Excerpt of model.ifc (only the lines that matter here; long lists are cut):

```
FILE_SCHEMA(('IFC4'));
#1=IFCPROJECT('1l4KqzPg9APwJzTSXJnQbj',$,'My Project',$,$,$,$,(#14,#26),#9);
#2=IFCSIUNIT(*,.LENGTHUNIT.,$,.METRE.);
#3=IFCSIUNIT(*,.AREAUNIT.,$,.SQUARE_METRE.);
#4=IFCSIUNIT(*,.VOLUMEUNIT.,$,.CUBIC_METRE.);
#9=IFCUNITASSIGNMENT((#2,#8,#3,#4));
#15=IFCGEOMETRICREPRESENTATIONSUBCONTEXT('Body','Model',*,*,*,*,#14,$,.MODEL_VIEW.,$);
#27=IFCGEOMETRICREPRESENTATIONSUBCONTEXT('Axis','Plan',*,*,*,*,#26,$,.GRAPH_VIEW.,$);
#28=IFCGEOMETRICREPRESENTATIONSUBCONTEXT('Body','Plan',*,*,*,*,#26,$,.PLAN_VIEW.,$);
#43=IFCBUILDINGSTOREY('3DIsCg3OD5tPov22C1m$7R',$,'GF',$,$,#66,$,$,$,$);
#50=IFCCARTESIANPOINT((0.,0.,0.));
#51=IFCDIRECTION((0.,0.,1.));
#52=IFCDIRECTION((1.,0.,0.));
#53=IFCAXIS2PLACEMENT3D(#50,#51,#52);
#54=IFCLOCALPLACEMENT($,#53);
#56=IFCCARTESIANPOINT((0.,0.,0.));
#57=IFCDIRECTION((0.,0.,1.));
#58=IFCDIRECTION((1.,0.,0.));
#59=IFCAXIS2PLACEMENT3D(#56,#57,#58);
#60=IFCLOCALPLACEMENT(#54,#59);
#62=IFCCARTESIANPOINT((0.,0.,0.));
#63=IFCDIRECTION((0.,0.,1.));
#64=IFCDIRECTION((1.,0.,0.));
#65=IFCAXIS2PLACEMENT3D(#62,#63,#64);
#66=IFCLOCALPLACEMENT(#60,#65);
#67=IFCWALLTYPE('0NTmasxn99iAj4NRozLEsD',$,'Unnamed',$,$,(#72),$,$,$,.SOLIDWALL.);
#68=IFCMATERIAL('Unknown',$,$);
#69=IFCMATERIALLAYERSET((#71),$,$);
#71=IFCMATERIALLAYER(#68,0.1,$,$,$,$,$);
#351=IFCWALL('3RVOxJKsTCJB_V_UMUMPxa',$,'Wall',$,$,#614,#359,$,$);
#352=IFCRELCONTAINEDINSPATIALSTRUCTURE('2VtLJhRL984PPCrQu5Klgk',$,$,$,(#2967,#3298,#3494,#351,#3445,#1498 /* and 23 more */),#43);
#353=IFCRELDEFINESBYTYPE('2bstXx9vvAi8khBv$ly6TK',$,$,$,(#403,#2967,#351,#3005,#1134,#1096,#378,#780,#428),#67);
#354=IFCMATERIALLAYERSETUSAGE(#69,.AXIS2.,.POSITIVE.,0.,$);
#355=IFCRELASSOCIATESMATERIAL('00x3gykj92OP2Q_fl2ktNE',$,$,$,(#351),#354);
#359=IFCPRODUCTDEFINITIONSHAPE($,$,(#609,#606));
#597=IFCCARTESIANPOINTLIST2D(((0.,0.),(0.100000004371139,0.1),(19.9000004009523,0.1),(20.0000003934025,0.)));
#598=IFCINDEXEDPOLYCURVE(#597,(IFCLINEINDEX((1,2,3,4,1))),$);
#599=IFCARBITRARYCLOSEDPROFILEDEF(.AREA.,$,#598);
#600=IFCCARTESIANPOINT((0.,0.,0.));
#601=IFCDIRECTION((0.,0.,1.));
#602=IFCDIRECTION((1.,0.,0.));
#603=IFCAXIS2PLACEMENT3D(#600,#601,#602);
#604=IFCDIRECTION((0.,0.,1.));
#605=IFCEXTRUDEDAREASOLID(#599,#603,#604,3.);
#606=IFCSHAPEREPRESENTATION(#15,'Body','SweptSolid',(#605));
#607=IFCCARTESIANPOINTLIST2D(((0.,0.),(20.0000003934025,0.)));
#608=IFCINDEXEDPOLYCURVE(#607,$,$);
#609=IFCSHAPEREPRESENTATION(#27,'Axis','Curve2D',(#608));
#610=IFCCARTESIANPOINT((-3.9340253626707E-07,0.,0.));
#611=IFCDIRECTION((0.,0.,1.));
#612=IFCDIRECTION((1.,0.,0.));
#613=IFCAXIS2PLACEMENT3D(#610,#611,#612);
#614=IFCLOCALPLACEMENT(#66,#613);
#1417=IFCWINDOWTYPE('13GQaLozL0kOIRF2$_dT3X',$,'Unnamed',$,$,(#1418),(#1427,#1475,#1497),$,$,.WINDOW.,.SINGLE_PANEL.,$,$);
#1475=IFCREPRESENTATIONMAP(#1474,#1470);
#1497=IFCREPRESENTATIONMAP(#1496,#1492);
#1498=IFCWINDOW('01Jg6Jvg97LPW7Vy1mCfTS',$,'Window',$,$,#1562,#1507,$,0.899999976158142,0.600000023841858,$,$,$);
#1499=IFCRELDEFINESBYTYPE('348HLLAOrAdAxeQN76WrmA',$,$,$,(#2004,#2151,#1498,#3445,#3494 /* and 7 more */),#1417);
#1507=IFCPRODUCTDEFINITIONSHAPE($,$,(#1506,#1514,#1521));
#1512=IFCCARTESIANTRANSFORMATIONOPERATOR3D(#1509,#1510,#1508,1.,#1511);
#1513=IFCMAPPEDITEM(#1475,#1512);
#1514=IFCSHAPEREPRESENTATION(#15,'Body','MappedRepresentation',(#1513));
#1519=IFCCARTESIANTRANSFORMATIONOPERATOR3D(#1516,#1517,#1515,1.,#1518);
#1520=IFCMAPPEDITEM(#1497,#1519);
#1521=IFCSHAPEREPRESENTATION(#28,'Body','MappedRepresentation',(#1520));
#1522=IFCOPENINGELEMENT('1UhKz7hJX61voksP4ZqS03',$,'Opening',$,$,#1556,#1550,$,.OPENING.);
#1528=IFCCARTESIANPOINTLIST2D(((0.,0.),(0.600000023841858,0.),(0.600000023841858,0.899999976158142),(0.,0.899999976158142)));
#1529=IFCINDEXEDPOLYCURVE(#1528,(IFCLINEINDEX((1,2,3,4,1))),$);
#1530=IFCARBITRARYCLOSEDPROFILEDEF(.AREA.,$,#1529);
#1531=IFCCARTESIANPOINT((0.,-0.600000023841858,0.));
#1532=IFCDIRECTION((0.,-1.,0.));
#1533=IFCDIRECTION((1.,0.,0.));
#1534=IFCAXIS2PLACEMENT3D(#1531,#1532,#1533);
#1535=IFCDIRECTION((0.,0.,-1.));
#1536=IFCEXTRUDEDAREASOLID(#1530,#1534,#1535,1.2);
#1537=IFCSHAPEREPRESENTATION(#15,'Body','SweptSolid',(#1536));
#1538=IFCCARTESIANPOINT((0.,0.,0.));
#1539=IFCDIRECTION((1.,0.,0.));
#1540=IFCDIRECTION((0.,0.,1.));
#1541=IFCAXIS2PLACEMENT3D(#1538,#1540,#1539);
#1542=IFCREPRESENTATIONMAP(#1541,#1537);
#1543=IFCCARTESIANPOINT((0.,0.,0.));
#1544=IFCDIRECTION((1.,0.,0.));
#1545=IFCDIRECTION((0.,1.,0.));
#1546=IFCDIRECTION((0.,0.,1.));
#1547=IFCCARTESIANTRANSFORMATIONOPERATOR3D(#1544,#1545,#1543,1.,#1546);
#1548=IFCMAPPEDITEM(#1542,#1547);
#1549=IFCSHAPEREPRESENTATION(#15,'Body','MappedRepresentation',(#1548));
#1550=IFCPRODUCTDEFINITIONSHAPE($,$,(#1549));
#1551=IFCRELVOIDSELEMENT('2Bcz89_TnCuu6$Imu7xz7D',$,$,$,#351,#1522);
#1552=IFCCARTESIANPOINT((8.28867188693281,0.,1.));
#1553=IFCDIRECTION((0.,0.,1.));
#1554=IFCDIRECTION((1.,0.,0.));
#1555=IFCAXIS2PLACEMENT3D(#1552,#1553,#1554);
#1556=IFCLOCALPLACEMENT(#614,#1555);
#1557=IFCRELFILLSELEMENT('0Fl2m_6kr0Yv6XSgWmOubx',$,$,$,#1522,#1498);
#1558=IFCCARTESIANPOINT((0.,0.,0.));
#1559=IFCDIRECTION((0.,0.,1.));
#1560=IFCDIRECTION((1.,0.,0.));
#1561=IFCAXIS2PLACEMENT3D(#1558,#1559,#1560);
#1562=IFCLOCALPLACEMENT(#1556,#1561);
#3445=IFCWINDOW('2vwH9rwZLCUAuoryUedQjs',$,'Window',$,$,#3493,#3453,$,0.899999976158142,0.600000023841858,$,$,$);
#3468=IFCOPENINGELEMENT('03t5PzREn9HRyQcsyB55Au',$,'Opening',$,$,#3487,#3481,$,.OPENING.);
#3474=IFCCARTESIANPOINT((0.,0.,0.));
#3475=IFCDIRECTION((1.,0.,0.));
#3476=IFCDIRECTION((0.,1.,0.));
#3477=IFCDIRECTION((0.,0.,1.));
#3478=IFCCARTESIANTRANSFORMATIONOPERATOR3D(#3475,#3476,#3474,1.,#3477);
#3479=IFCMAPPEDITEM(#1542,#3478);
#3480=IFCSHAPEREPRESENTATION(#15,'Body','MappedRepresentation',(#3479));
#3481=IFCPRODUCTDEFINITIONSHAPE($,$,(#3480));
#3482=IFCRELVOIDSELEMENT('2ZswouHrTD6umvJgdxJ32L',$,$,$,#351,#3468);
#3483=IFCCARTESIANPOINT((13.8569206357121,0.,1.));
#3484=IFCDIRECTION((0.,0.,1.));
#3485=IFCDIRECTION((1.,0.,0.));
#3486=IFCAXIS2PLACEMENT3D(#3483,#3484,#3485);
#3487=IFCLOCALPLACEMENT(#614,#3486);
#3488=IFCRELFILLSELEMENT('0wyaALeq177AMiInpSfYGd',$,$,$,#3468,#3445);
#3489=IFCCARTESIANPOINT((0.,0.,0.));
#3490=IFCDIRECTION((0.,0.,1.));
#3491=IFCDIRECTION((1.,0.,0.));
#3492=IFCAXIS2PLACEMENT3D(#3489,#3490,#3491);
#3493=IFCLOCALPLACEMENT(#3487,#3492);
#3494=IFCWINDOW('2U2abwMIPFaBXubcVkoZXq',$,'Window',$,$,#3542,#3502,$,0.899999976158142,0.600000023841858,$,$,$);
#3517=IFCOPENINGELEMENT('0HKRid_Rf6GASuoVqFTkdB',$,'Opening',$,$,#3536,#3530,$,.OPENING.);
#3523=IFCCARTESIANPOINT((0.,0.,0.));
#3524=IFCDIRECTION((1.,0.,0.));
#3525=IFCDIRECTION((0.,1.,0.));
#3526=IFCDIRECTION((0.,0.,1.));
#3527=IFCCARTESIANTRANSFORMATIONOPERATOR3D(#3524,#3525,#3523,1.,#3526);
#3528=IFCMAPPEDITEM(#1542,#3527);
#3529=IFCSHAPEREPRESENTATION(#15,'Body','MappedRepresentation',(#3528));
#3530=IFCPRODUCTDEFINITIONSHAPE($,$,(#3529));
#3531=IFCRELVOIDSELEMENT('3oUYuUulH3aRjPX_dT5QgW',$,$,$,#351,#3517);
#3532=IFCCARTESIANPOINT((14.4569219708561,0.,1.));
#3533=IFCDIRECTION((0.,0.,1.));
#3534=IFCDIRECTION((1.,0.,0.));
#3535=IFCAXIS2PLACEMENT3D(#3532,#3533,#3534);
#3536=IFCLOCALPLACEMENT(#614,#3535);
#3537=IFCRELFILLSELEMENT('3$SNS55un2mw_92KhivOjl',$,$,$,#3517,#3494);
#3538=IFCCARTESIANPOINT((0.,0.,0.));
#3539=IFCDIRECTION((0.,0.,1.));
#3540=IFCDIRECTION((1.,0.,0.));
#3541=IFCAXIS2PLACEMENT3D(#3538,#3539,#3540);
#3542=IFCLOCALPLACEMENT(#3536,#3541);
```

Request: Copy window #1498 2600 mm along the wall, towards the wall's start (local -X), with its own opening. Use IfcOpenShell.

```python
import ifcopenshell
import ifcopenshell.api.feature
import ifcopenshell.api.geometry
import ifcopenshell.api.root
import ifcopenshell.geom
import ifcopenshell.util.element
import ifcopenshell.util.placement
import ifcopenshell.util.shape

model = ifcopenshell.open("model.ifc")
settings = ifcopenshell.geom.settings()


def volume(element):
    """Net volume in cubic metres, openings subtracted."""
    shape = ifcopenshell.geom.create_shape(settings, element)
    return ifcopenshell.util.shape.get_volume(shape.geometry)


window = model.by_guid("01Jg6Jvg97LPW7Vy1mCfTS")
opening = window.FillsVoids[0].RelatingOpeningElement
wall = opening.VoidsElements[0].RelatingBuildingElement
before = volume(wall)
shift = ifcopenshell.util.placement.get_local_placement(wall.ObjectPlacement)[:3, 0] * -2.6

# copy_class copies the void relationship, type, container and properties, but no geometry.
new_opening = ifcopenshell.api.root.copy_class(model, product=opening)
new_opening.Representation = ifcopenshell.util.element.copy_deep(
    model, opening.Representation, exclude=["IfcGeometricRepresentationContext", "IfcRepresentationMap"]
)
new_window = ifcopenshell.api.root.copy_class(model, product=window)
new_window.Representation = ifcopenshell.util.element.copy_deep(
    model, window.Representation, exclude=["IfcGeometricRepresentationContext", "IfcRepresentationMap"]
)
ifcopenshell.api.feature.add_filling(model, opening=new_opening, element=new_window)

for old, new in ((opening, new_opening), (window, new_window)):
    matrix = ifcopenshell.util.placement.get_local_placement(old.ObjectPlacement)
    matrix[:3, 3] += shift
    ifcopenshell.api.geometry.edit_object_placement(model, product=new, matrix=matrix, is_si=False)

after = volume(wall)

print(f"wall volume {before:.3f} -> {after:.3f} m3")

model.write("model_v2.ifc")
```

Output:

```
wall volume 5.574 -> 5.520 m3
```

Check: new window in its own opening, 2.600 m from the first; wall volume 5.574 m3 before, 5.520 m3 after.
